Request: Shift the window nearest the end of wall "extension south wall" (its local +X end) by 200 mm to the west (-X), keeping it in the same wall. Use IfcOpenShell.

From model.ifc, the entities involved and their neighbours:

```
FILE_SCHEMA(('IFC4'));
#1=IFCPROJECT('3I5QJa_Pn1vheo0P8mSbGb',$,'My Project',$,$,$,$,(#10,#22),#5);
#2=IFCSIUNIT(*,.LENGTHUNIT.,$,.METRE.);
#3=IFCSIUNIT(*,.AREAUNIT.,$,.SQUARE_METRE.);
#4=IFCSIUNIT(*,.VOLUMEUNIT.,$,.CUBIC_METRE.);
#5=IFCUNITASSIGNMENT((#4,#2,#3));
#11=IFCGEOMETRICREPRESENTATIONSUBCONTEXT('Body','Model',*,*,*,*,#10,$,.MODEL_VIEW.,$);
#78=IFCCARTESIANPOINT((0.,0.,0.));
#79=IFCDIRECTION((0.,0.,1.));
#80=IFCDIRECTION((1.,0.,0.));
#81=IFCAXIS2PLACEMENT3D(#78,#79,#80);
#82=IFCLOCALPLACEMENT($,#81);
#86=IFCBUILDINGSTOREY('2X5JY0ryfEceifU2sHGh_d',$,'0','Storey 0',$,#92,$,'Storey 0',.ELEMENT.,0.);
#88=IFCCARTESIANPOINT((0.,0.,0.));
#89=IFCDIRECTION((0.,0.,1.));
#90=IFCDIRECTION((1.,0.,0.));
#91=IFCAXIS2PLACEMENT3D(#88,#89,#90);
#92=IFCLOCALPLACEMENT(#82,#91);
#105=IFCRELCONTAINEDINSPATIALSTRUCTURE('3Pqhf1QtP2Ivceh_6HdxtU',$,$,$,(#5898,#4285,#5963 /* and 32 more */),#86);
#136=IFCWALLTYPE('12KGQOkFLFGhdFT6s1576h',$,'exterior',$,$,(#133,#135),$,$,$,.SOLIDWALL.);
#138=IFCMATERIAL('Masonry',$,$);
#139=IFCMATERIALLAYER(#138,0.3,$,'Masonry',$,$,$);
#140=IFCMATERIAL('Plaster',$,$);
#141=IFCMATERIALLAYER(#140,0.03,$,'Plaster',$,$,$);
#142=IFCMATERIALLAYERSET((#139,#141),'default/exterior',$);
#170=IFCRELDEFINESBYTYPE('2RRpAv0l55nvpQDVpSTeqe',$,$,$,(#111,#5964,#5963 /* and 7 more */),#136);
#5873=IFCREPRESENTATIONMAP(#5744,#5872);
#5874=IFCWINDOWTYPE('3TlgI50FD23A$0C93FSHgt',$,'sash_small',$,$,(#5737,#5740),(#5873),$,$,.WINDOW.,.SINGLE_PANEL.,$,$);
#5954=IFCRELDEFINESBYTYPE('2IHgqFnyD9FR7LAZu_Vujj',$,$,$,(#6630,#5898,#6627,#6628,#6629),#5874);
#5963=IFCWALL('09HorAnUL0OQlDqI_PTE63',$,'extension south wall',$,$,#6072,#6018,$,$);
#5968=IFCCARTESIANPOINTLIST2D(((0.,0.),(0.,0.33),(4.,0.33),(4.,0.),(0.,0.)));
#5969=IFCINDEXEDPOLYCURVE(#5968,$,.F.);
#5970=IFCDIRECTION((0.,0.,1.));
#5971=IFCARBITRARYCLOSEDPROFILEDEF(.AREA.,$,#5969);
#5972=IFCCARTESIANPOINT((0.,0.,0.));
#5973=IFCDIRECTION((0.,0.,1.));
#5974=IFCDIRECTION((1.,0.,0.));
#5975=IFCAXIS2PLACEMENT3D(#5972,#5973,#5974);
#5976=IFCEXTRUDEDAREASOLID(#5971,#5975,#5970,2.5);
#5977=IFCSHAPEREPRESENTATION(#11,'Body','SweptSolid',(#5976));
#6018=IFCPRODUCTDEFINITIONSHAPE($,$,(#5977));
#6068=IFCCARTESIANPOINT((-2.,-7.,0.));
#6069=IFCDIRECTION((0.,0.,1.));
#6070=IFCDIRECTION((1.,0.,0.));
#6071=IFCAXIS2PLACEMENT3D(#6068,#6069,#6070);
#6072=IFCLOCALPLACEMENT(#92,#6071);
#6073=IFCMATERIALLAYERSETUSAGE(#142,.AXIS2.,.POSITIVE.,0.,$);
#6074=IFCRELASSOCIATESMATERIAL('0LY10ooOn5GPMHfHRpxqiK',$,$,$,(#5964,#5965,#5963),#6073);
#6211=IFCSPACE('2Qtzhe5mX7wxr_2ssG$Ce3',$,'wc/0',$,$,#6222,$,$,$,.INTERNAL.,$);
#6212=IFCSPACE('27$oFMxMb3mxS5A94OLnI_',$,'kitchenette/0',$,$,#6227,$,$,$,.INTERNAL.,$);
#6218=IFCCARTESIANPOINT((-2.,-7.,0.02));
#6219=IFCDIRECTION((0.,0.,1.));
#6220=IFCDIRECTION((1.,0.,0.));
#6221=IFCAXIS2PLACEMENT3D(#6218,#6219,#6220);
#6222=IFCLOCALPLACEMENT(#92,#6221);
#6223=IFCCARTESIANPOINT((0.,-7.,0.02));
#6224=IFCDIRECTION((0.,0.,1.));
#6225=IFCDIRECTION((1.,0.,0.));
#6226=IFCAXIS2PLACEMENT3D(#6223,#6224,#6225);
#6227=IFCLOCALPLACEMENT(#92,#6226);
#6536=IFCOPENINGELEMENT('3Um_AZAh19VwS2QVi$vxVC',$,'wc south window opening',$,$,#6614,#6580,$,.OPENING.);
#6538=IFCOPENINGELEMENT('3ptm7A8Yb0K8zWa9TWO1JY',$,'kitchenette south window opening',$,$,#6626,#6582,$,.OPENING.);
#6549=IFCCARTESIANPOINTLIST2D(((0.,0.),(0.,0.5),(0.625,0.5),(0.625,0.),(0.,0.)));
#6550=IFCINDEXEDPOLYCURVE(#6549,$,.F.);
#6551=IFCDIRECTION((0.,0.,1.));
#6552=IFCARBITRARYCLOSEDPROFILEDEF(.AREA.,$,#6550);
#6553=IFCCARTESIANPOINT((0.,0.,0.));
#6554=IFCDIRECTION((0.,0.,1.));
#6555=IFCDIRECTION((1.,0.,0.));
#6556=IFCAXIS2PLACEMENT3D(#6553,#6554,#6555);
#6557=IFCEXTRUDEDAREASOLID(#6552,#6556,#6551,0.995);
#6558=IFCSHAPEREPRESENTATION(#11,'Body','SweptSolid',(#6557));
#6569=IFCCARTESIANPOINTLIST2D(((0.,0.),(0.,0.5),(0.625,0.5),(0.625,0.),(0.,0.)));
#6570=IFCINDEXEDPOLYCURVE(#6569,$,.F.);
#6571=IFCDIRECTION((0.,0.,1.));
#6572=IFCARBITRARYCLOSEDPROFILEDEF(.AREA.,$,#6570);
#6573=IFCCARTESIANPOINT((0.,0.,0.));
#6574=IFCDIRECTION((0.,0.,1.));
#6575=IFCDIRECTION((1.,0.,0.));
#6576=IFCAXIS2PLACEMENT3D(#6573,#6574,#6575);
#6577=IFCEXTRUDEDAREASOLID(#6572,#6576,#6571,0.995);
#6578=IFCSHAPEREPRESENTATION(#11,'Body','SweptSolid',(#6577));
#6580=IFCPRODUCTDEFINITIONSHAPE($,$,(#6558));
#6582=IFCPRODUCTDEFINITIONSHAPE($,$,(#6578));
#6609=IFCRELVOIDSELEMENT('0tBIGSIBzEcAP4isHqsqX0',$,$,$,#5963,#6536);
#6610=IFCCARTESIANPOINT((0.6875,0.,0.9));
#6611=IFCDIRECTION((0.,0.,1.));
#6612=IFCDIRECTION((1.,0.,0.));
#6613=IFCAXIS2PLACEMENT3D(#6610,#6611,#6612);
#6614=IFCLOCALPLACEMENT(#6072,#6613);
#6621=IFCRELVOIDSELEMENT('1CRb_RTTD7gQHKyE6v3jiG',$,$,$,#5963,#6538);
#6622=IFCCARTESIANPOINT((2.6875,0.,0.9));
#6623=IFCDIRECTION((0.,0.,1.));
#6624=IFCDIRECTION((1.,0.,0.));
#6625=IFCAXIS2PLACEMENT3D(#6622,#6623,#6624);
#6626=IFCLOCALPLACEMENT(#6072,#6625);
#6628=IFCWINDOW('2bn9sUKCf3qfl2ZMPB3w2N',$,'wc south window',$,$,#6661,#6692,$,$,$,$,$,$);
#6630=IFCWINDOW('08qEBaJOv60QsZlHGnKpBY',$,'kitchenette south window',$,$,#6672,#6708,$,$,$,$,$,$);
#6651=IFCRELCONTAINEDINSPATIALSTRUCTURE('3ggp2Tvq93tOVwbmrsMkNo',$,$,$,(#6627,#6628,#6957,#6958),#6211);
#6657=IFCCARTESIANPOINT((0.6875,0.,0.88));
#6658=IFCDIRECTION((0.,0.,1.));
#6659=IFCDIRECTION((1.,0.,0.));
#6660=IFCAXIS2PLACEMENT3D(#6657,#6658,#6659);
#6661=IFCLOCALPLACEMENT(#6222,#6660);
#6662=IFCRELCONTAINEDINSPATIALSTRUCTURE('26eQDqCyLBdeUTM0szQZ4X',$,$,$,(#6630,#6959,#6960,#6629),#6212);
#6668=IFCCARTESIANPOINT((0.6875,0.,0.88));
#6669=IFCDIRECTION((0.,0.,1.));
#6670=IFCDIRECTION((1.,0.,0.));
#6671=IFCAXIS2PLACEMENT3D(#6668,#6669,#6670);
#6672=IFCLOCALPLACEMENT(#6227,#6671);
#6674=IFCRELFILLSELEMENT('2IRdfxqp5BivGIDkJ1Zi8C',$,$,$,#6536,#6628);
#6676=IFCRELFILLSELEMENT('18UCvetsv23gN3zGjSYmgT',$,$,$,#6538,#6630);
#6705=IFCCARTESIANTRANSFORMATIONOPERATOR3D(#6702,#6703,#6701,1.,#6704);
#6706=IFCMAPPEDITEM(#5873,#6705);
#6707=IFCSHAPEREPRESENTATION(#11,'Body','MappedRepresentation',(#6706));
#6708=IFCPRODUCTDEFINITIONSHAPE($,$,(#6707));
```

```python
import ifcopenshell
import ifcopenshell.api.geometry
import ifcopenshell.util.placement
import ifcopenshell.util.unit

model = ifcopenshell.open("model.ifc")
unit_scale = ifcopenshell.util.unit.calculate_unit_scale(model)

window = model.by_id(6630)
opening = window.FillsVoids[0].RelatingOpeningElement
wall = opening.VoidsElements[0].RelatingBuildingElement

wall_matrix = ifcopenshell.util.placement.get_local_placement(wall.ObjectPlacement)
shift = wall_matrix[:3, 0] * -0.2 / unit_scale
before = ifcopenshell.util.placement.get_local_placement(window.ObjectPlacement)[:3, 3].copy()

# The window is not placed relative to its opening, so move both.
for product in (opening, window):
    matrix = ifcopenshell.util.placement.get_local_placement(product.ObjectPlacement)
    matrix[:3, 3] += shift
    ifcopenshell.api.geometry.edit_object_placement(model, product=product, matrix=matrix, is_si=False)

after = ifcopenshell.util.placement.get_local_placement(window.ObjectPlacement)[:3, 3]
print("window moved by", (after - before).round(3) + 0.0)

model.write("model-out.ifc")
```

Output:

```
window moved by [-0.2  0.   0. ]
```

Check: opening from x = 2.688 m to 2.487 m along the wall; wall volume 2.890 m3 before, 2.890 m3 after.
